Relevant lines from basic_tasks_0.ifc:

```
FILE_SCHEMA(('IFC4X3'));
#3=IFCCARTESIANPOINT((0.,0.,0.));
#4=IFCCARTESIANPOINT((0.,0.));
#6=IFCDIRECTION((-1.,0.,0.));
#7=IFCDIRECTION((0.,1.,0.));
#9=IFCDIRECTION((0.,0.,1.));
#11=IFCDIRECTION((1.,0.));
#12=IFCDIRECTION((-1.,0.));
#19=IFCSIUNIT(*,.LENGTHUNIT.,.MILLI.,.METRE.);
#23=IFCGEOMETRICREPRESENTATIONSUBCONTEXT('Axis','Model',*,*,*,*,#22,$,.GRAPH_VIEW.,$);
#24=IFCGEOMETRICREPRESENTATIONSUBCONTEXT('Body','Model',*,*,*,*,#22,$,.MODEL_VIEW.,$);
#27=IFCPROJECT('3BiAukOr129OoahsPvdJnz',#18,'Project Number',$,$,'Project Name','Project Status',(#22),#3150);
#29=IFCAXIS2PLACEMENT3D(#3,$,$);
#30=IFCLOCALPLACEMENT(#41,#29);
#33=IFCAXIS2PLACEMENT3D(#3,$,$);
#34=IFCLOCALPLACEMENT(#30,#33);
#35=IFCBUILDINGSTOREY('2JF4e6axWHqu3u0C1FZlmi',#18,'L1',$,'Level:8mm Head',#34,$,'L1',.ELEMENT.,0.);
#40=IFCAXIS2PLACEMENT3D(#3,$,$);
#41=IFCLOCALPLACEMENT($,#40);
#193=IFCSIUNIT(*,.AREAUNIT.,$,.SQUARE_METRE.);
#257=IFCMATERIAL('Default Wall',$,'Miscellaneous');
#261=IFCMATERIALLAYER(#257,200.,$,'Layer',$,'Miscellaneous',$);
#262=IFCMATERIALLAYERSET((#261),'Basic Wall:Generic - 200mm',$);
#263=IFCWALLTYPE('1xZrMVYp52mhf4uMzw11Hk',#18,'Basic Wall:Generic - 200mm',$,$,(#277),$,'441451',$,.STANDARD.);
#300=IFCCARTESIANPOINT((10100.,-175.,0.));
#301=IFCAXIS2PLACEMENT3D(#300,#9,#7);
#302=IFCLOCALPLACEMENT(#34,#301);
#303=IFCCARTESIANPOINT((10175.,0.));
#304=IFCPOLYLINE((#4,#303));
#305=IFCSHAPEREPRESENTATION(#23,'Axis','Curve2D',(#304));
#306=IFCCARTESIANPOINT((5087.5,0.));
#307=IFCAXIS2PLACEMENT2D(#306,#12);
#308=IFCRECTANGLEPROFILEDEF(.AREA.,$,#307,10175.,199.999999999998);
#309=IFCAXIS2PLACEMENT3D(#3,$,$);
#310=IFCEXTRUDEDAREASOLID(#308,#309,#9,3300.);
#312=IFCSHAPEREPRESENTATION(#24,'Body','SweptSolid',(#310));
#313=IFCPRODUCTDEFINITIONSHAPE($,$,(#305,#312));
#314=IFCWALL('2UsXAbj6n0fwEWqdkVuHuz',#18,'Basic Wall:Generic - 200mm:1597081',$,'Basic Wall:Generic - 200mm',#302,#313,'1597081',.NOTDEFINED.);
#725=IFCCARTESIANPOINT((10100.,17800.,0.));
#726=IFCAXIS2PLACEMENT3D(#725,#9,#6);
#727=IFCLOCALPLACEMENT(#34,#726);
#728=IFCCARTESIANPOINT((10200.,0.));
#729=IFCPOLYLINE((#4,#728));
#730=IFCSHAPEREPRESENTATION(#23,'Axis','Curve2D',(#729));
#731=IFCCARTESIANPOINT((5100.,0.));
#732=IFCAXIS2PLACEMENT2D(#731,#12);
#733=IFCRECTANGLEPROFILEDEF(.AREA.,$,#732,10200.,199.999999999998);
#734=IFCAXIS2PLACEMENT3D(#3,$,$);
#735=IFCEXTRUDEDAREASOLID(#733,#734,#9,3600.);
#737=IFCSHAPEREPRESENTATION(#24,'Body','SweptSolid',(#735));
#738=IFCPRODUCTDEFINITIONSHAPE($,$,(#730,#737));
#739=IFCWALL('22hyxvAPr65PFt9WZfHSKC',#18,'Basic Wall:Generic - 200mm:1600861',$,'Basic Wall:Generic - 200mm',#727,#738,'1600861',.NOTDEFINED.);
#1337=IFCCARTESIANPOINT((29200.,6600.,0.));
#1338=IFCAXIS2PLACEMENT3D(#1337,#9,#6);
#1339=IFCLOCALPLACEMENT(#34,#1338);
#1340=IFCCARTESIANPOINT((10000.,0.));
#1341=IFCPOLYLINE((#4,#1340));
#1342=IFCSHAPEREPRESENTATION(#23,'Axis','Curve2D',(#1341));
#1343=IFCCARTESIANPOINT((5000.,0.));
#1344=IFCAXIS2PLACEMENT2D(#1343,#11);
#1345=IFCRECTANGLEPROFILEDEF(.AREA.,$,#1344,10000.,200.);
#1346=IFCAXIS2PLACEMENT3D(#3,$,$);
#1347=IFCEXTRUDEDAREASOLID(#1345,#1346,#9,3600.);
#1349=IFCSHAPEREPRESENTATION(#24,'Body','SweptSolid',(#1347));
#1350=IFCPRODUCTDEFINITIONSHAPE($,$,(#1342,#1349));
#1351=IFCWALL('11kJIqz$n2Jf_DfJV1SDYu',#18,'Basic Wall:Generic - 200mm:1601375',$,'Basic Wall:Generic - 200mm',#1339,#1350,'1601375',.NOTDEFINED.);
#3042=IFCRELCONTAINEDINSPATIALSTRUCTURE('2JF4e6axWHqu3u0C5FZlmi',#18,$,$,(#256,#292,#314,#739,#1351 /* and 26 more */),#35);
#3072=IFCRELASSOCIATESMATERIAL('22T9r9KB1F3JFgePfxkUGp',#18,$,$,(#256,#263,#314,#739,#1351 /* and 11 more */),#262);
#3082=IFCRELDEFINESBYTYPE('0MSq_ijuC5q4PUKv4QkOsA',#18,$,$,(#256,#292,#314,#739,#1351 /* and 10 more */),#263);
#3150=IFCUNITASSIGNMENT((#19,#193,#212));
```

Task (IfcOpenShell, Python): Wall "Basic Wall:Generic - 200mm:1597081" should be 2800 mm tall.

```python
import ifcopenshell
import ifcopenshell.geom
import ifcopenshell.util.representation
import ifcopenshell.util.shape

model = ifcopenshell.open("basic_tasks_0.ifc")
settings = ifcopenshell.geom.settings()


def volume(element):
    """Net volume in cubic metres, openings subtracted."""
    shape = ifcopenshell.geom.create_shape(settings, element)
    return ifcopenshell.util.shape.get_volume(shape.geometry)


wall = model.by_guid("2UsXAbj6n0fwEWqdkVuHuz")
before = volume(wall)

body = ifcopenshell.util.representation.get_representation(wall, "Model", "Body")
solid = body.Items[0]
old_height = solid.Depth
solid.Depth = 2800.0
after = volume(wall)

print(f"height {old_height:g} -> {solid.Depth:g}, volume {before:.3f} -> {after:.3f} m3")

model.write("basic_tasks_0_updated.ifc")
```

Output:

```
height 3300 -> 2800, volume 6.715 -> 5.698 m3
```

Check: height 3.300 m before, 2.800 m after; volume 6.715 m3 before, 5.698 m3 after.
